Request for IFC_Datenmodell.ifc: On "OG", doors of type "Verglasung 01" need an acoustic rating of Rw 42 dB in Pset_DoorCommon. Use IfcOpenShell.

First a look at what the model holds.

```python
import ifcopenshell
import ifcopenshell.util.element

model = ifcopenshell.open("IFC_Datenmodell.ifc")
print(model.schema)
storey = next(s for s in model.by_type("IfcBuildingStorey") if s.Name == "OG")
doors = [e for e in ifcopenshell.util.element.get_decomposition(storey) if e.is_a("IfcDoor")]
seen = {}
for e in doors:
    element_type = ifcopenshell.util.element.get_type(e)
    key = (element_type.Name if element_type != e and element_type else None, ifcopenshell.util.element.get_pset(e, "Pset_DoorCommon", "AcousticRating"))
    seen[key] = seen.get(key, 0) + 1
for (name, value), count in sorted(seen.items(), key=str):
    print(count, "x", name, "|", value)
```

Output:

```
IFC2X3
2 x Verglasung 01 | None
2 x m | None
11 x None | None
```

```python
import ifcopenshell
import ifcopenshell.api.pset
import ifcopenshell.util.element

model = ifcopenshell.open("IFC_Datenmodell.ifc")

storey = next(s for s in model.by_type("IfcBuildingStorey") if s.Name == "OG")
doors = [e for e in ifcopenshell.util.element.get_decomposition(storey) if e.is_a("IfcDoor")]

count = 0
for e in doors:
    element_type = ifcopenshell.util.element.get_type(e)
    if element_type in (None, e) or element_type.Name != "Verglasung 01":
        continue
    # add_pset returns the element's existing set when there is one.
    pset = ifcopenshell.api.pset.add_pset(model, product=e, name="Pset_DoorCommon")
    ifcopenshell.api.pset.edit_pset(model, pset=pset, properties={"AcousticRating": "Rw 42 dB"})
    count += 1

print(count, "doors updated")

model.write("IFC_Datenmodell_edited.ifc")
```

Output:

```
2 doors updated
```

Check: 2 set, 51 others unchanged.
